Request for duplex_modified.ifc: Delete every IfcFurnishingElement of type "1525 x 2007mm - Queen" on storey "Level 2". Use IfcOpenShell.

First a look at what the model holds.

```python
import ifcopenshell
import ifcopenshell.util.element

model = ifcopenshell.open("duplex_modified.ifc")
print(model.schema)
storey = next(s for s in model.by_type("IfcBuildingStorey") if s.Name == "Level 2")
furniture = [e for e in ifcopenshell.util.element.get_decomposition(storey) if e.is_a("IfcFurnishingElement")]
seen = {}
for e in furniture:
    element_type = ifcopenshell.util.element.get_type(e)
    name = element_type.Name if element_type not in (None, e) else None
    seen[name] = seen.get(name, 0) + 1
for name, count in sorted(seen.items(), key=str):
    print(count, "x", name)
```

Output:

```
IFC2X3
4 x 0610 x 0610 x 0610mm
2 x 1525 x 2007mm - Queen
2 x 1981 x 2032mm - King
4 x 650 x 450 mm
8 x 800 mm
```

```python
import ifcopenshell
import ifcopenshell.api.root
import ifcopenshell.util.element

model = ifcopenshell.open("duplex_modified.ifc")

storey = next(s for s in model.by_type("IfcBuildingStorey") if s.Name == "Level 2")
furniture = [e for e in ifcopenshell.util.element.get_decomposition(storey) if e.is_a("IfcFurnishingElement")]
targets = [e for e in furniture if (t := ifcopenshell.util.element.get_type(e)) not in (None, e) and t.Name == "1525 x 2007mm - Queen"]

for e in targets:
    ifcopenshell.api.root.remove_product(model, product=e)
print(len(targets), "removed")

model.write("duplex_modified_edited.ifc")
```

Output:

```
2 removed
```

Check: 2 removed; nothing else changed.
